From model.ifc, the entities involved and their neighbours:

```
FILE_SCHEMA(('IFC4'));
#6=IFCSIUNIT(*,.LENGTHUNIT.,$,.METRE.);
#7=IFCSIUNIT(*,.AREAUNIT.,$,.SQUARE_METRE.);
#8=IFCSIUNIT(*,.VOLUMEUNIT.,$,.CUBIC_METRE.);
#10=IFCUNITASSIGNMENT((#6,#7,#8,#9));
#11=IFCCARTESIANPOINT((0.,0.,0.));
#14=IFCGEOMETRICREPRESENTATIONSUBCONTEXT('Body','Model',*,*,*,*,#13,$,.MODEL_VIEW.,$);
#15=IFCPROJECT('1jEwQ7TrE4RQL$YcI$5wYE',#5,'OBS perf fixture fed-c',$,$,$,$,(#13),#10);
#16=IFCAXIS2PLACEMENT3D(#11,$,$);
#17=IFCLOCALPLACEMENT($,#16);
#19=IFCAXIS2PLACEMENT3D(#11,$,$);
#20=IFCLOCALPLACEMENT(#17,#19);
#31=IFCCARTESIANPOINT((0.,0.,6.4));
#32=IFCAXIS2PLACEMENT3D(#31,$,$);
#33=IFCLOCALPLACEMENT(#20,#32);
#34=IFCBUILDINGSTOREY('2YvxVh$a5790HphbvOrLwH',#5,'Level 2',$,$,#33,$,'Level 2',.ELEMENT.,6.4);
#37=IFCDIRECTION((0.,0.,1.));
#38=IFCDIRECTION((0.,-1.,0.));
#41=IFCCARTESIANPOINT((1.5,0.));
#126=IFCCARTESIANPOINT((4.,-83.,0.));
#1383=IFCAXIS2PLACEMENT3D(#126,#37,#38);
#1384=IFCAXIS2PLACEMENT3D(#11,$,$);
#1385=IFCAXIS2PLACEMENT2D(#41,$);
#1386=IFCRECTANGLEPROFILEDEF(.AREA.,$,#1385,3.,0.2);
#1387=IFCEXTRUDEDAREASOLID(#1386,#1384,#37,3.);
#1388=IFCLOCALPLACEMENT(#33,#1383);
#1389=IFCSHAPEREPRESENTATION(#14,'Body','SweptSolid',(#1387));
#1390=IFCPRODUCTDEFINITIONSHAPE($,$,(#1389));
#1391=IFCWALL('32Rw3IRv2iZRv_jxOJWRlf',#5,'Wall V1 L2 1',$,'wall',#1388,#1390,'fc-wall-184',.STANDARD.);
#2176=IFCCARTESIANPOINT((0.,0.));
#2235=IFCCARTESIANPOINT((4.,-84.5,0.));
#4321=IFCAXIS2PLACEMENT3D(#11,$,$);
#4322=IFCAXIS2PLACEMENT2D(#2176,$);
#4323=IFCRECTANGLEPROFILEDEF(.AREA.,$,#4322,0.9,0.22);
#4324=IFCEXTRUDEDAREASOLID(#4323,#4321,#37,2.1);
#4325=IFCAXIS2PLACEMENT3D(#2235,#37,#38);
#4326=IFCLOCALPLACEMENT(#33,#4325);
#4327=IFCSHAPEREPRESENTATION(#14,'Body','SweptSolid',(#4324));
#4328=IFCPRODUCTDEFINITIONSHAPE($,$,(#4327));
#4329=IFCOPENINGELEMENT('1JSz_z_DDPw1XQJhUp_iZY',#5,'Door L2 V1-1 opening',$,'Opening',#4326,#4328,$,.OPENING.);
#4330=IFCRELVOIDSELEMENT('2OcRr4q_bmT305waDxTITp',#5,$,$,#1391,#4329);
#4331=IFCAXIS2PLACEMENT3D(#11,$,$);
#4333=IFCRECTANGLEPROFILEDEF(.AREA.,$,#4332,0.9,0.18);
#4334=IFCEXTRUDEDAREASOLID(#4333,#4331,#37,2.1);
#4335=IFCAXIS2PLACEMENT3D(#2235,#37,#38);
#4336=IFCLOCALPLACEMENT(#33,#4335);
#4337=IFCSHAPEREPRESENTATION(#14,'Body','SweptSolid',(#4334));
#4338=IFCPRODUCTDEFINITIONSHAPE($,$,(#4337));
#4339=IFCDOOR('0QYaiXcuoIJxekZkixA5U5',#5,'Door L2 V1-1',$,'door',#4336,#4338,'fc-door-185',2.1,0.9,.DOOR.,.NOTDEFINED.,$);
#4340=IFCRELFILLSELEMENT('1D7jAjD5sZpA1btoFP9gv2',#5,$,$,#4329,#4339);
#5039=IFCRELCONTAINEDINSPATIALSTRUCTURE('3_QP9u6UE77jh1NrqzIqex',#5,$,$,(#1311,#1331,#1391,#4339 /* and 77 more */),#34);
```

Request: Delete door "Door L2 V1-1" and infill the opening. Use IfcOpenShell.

```python
import ifcopenshell
import ifcopenshell.api.feature
import ifcopenshell.api.root
import ifcopenshell.geom
import ifcopenshell.util.shape

model = ifcopenshell.open("model.ifc")
settings = ifcopenshell.geom.settings()


def volume(element):
    """Net volume in cubic metres, openings subtracted."""
    shape = ifcopenshell.geom.create_shape(settings, element)
    return ifcopenshell.util.shape.get_volume(shape.geometry)


door = model.by_guid("0QYaiXcuoIJxekZkixA5U5")
opening = door.FillsVoids[0].RelatingOpeningElement
wall = opening.VoidsElements[0].RelatingBuildingElement
before = volume(wall)

ifcopenshell.api.root.remove_product(model, product=door)
ifcopenshell.api.feature.remove_feature(model, feature=opening)

after = volume(wall)

print(f"wall volume {before:.3f} -> {after:.3f} m3")

model.write("model_edited.ifc")
```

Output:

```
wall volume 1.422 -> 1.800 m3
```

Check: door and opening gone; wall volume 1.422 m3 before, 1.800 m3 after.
